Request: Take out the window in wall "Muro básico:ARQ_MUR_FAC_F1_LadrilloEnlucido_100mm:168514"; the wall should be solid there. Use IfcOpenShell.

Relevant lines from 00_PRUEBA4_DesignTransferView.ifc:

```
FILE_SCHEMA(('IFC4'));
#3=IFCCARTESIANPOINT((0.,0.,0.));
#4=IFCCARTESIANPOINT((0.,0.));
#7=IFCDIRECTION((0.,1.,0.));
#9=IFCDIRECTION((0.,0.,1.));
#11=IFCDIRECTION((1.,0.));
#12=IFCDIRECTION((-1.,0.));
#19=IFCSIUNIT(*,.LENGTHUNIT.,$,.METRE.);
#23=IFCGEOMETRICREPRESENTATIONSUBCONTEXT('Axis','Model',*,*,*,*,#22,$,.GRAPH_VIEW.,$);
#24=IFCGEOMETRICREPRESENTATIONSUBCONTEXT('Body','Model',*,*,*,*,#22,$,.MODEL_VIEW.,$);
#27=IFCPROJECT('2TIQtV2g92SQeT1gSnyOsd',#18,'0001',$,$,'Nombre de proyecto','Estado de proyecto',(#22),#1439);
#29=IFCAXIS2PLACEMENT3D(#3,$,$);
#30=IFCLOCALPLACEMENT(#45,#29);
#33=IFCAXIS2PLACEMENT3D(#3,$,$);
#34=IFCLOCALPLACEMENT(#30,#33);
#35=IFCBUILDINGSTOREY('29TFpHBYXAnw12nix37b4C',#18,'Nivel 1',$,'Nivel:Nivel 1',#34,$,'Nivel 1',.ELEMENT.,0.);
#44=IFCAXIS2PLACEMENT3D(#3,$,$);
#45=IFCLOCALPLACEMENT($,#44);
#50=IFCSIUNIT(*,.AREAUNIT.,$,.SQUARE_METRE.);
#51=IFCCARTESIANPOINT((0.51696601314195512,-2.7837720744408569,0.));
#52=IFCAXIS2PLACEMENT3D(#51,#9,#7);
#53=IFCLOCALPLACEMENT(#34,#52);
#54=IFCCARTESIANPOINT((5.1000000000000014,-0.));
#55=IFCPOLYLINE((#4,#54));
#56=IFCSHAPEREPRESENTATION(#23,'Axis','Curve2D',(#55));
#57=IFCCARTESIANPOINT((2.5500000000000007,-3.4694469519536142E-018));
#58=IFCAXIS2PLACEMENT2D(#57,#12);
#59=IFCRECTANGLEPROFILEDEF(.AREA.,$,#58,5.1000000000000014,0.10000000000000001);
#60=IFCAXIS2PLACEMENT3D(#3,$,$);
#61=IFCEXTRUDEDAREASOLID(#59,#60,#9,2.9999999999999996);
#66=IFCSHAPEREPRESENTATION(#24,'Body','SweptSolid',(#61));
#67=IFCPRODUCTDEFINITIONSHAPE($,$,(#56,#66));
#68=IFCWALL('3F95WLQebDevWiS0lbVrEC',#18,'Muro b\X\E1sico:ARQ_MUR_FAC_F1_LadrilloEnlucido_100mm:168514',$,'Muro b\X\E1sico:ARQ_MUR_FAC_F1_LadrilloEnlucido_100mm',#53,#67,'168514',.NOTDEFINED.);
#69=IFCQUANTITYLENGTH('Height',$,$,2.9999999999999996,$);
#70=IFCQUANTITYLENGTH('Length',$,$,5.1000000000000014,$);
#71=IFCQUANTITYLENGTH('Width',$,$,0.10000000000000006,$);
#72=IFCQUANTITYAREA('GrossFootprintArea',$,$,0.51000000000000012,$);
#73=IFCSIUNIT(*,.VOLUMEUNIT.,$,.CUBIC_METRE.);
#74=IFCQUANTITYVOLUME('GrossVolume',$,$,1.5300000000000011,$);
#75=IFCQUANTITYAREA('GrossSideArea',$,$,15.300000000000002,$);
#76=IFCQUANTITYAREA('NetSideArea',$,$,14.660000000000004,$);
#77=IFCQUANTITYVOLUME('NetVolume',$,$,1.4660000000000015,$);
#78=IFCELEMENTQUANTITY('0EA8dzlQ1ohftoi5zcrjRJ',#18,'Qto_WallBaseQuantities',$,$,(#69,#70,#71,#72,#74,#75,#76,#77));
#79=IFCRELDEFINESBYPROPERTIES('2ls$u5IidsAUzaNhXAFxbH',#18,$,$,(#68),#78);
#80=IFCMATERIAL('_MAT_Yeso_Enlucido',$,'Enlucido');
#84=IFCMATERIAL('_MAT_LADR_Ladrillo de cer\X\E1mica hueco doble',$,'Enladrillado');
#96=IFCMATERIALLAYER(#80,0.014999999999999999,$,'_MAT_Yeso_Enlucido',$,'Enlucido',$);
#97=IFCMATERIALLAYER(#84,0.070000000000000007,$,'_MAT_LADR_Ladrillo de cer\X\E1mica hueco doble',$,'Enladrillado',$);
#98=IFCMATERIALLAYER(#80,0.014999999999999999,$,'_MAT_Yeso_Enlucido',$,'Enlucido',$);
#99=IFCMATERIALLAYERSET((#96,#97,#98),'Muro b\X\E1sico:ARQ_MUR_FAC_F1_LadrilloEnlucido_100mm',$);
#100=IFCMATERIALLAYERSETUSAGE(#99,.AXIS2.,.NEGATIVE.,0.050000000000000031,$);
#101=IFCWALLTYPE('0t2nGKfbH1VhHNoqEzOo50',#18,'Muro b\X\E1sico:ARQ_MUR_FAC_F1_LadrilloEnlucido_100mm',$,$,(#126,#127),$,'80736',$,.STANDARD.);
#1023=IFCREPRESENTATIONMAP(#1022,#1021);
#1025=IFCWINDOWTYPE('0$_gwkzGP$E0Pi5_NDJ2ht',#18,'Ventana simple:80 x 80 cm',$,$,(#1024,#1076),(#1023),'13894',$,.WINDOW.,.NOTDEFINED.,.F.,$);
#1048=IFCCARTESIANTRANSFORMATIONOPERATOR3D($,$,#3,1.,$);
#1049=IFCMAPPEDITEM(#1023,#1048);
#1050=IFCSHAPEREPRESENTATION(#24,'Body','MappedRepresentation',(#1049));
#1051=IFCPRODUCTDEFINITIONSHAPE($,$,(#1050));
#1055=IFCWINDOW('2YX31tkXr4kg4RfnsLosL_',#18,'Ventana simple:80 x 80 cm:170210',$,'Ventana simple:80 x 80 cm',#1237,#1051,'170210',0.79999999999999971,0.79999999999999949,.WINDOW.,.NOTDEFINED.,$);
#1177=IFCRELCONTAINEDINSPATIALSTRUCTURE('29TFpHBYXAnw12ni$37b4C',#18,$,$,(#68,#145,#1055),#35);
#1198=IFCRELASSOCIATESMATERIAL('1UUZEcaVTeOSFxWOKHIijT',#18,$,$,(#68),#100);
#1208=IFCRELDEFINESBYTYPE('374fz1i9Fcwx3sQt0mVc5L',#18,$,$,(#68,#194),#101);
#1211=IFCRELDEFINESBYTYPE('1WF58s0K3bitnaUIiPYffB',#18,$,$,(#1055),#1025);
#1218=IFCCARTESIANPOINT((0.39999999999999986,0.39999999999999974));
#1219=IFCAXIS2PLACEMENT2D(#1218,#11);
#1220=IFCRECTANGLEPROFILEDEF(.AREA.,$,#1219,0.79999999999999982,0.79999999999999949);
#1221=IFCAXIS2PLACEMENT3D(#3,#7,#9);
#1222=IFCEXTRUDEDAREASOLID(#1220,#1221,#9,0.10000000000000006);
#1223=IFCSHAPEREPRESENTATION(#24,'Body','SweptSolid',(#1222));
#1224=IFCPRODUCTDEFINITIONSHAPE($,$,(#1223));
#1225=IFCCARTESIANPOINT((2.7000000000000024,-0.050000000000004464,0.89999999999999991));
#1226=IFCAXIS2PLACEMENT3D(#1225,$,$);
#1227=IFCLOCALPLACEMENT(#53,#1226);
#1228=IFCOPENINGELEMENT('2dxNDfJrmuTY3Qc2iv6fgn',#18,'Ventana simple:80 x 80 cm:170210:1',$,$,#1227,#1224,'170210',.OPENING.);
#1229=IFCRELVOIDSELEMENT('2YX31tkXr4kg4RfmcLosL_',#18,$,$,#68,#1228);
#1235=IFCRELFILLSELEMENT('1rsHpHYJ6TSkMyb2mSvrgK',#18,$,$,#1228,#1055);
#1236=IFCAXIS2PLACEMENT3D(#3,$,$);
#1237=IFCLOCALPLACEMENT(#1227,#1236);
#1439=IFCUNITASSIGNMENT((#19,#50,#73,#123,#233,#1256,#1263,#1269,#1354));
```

```python
import ifcopenshell
import ifcopenshell.api.feature
import ifcopenshell.api.pset
import ifcopenshell.api.root
import ifcopenshell.geom
import ifcopenshell.util.element
import ifcopenshell.util.shape
import ifcopenshell.util.unit

model = ifcopenshell.open("00_PRUEBA4_DesignTransferView.ifc")
area_scale = ifcopenshell.util.unit.calculate_unit_scale(model, "AREAUNIT")
volume_scale = ifcopenshell.util.unit.calculate_unit_scale(model, "VOLUMEUNIT")
settings = ifcopenshell.geom.settings()


def volume(element):
    """Net volume in cubic metres, openings subtracted."""
    shape = ifcopenshell.geom.create_shape(settings, element)
    return ifcopenshell.util.shape.get_volume(shape.geometry)


window = model.by_guid("2YX31tkXr4kg4RfnsLosL_")
opening = window.FillsVoids[0].RelatingOpeningElement
wall = opening.VoidsElements[0].RelatingBuildingElement
before = volume(wall)

ifcopenshell.api.root.remove_product(model, product=window)
ifcopenshell.api.feature.remove_feature(model, feature=opening)

after = volume(wall)
thickness = 0.1  # wall thickness in metres

# Update the wall's stored quantities.
qto = model.by_id(ifcopenshell.util.element.get_pset(wall, "Qto_WallBaseQuantities", should_inherit=False)["id"])
ifcopenshell.api.pset.edit_qto(model, qto=qto, properties={
    "NetSideArea": after / thickness / area_scale,
    "NetVolume": after / volume_scale,
})

print(f"wall volume {before:.3f} -> {after:.3f} m3")

model.write("00_PRUEBA4_DesignTransferView_edited.ifc")
```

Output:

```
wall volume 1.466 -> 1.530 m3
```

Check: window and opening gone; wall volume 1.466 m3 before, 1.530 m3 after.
